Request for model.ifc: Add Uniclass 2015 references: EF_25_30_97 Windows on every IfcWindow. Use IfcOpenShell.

First a look at what the model holds.

```python
import ifcopenshell

model = ifcopenshell.open("model.ifc")
print(model.schema)
print("classifications:", [c.Name for c in model.by_type("IfcClassification")])
for ifc_class in ("IfcDoor", "IfcRoof", "IfcStair", "IfcWall", "IfcWindow"):
    print(ifc_class, len(model.by_type(ifc_class)))
```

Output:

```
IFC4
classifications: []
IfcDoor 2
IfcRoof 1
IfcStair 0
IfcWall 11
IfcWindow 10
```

```python
import ifcopenshell
import ifcopenshell.api.classification

model = ifcopenshell.open("model.ifc")

system = ifcopenshell.api.classification.add_classification(model, classification="Uniclass 2015")

codes = {
    "IfcWindow": ("EF_25_30_97", "Windows"),
}
for ifc_class, (code, name) in codes.items():
    products = model.by_type(ifc_class)
    ifcopenshell.api.classification.add_reference(
        model, products=products, classification=system, identification=code, name=name
    )
    print(code, len(products))

model.write("model_updated.ifc")
```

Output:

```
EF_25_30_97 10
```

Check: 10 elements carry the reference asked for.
